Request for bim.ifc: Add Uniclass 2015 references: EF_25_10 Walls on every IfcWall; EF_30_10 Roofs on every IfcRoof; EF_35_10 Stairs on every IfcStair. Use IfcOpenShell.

First a look at what the model holds.

```python
import ifcopenshell

model = ifcopenshell.open("bim.ifc")
print(model.schema)
print("classifications:", [c.Name for c in model.by_type("IfcClassification")])
for ifc_class in ("IfcDoor", "IfcRoof", "IfcStair", "IfcWall", "IfcWindow"):
    print(ifc_class, len(model.by_type(ifc_class)))
```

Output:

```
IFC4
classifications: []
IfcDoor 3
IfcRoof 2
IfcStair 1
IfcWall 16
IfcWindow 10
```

```python
import ifcopenshell
import ifcopenshell.api.classification

model = ifcopenshell.open("bim.ifc")

system = ifcopenshell.api.classification.add_classification(model, classification="Uniclass 2015")

codes = {
    "IfcWall": ("EF_25_10", "Walls"),
    "IfcRoof": ("EF_30_10", "Roofs"),
    "IfcStair": ("EF_35_10", "Stairs"),
}
for ifc_class, (code, name) in codes.items():
    products = model.by_type(ifc_class)
    ifcopenshell.api.classification.add_reference(
        model, products=products, classification=system, identification=code, name=name
    )
    print(code, len(products))

model.write("bim_v2.ifc")
```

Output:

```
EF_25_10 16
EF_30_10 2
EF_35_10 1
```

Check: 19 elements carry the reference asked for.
